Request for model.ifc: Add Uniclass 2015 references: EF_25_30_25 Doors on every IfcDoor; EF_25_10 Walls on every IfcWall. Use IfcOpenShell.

First a look at what the model holds.

```python
import ifcopenshell

model = ifcopenshell.open("model.ifc")
print(model.schema)
print("classifications:", [c.Name for c in model.by_type("IfcClassification")])
for ifc_class in ("IfcDoor", "IfcRoof", "IfcStair", "IfcWall", "IfcWindow"):
    print(ifc_class, len(model.by_type(ifc_class)))
```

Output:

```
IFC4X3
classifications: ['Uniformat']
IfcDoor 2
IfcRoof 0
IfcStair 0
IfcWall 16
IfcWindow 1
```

```python
import ifcopenshell
import ifcopenshell.api.classification

model = ifcopenshell.open("model.ifc")

system = ifcopenshell.api.classification.add_classification(model, classification="Uniclass 2015")

codes = {
    "IfcDoor": ("EF_25_30_25", "Doors"),
    "IfcWall": ("EF_25_10", "Walls"),
}
for ifc_class, (code, name) in codes.items():
    products = model.by_type(ifc_class)
    ifcopenshell.api.classification.add_reference(
        model, products=products, classification=system, identification=code, name=name
    )
    print(code, len(products))

model.write("model_edited.ifc")
```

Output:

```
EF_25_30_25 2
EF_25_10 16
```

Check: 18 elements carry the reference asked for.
